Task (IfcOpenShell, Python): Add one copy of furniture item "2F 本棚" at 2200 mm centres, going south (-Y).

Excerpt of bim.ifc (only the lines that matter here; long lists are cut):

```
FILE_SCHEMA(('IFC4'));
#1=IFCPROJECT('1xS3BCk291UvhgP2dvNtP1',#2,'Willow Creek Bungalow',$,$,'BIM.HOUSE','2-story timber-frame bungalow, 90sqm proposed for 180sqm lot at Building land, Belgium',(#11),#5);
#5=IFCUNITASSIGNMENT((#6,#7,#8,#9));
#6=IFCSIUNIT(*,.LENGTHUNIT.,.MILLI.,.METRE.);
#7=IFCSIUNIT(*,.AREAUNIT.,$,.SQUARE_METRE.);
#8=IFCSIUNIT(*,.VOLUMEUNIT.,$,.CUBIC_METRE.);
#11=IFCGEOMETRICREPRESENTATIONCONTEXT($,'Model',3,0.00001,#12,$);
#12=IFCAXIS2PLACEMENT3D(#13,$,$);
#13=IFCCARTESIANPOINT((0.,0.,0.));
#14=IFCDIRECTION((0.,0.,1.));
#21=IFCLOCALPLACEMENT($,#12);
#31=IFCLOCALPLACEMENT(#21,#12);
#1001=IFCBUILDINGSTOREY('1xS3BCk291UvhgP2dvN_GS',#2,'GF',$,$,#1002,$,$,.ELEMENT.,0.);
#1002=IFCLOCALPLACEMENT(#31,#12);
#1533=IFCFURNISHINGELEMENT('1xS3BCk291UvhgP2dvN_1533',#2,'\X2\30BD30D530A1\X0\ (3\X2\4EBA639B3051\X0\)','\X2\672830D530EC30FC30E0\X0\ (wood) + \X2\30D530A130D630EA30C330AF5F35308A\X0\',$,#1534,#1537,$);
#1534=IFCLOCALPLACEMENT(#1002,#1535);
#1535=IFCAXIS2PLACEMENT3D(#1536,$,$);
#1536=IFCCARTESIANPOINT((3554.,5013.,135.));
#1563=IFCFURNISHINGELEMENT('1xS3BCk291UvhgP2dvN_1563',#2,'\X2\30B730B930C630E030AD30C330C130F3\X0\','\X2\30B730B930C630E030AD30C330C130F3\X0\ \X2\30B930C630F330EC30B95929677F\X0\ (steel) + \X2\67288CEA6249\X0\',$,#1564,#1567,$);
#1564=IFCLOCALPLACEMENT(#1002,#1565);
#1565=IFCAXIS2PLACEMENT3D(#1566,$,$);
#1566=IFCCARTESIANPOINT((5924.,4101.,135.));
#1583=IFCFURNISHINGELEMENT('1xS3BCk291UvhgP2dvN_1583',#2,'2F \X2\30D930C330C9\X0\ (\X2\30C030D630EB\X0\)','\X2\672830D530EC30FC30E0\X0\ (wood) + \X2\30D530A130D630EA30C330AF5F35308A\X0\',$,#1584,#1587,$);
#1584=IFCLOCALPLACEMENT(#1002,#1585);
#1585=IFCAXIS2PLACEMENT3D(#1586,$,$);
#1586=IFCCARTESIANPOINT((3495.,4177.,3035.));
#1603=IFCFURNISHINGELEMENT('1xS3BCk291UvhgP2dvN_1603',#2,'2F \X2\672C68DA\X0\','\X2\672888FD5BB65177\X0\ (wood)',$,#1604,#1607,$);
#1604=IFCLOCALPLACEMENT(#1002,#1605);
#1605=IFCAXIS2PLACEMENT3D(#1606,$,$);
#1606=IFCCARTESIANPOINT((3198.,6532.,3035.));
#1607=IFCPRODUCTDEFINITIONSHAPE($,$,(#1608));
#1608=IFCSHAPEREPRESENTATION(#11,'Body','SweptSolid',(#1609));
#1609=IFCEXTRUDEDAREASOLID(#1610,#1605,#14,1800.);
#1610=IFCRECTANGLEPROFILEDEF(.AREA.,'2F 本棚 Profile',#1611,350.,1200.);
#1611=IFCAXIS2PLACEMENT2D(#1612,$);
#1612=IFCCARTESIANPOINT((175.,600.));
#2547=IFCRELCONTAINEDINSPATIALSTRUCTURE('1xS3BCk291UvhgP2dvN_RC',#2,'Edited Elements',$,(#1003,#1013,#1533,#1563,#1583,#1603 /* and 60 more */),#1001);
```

```python
import numpy as np
import ifcopenshell
import ifcopenshell.api.geometry
import ifcopenshell.api.root
import ifcopenshell.util.element
import ifcopenshell.util.placement
import ifcopenshell.util.unit

model = ifcopenshell.open("bim.ifc")
unit_scale = ifcopenshell.util.unit.calculate_unit_scale(model)


def reuse_history(source, copy):
    """copy_class also copies each property set's owner history, people and application; keep the originals."""
    for rel in copy.IsDefinedBy:
        if rel.is_a("IfcRelDefinesByProperties") and (history := rel.RelatingPropertyDefinition.OwnerHistory):
            rel.RelatingPropertyDefinition.OwnerHistory = source.OwnerHistory
            ifcopenshell.util.element.remove_deep2(model, history)


source = model.by_guid("1xS3BCk291UvhgP2dvN_1603")
base = ifcopenshell.util.placement.get_local_placement(source.ObjectPlacement)
step = np.array([0.0, -1.0, 0.0]) * 2.2 / unit_scale

for i in range(1, 2):
    copy = ifcopenshell.api.root.copy_class(model, product=source)
    copy.Representation = ifcopenshell.util.element.copy_deep(
        model, source.Representation, exclude=["IfcGeometricRepresentationContext", "IfcRepresentationMap"]
    )
    reuse_history(source, copy)
    matrix = base.copy()
    matrix[:3, 3] += i * step
    print("added at", matrix[:3, 3].round(3) + 0.0)
    ifcopenshell.api.geometry.edit_object_placement(model, product=copy, matrix=matrix, is_si=False)

model.write("bim-out.ifc")
```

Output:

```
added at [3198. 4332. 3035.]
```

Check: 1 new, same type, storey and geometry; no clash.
